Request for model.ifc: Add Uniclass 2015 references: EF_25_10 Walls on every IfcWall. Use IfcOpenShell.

First a look at what the model holds.

```python
import ifcopenshell

model = ifcopenshell.open("model.ifc")
print(model.schema)
print("classifications:", [c.Name for c in model.by_type("IfcClassification")])
for ifc_class in ("IfcDoor", "IfcRoof", "IfcStair", "IfcWall", "IfcWindow"):
    print(ifc_class, len(model.by_type(ifc_class)))
```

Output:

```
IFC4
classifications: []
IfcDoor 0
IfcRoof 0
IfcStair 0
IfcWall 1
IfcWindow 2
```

```python
import ifcopenshell
import ifcopenshell.api.classification

model = ifcopenshell.open("model.ifc")

system = ifcopenshell.api.classification.add_classification(model, classification="Uniclass 2015")

codes = {
    "IfcWall": ("EF_25_10", "Walls"),
}
for ifc_class, (code, name) in codes.items():
    products = model.by_type(ifc_class)
    ifcopenshell.api.classification.add_reference(
        model, products=products, classification=system, identification=code, name=name
    )
    print(code, len(products))

model.write("model_edited.ifc")
```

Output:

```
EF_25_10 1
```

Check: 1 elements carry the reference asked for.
